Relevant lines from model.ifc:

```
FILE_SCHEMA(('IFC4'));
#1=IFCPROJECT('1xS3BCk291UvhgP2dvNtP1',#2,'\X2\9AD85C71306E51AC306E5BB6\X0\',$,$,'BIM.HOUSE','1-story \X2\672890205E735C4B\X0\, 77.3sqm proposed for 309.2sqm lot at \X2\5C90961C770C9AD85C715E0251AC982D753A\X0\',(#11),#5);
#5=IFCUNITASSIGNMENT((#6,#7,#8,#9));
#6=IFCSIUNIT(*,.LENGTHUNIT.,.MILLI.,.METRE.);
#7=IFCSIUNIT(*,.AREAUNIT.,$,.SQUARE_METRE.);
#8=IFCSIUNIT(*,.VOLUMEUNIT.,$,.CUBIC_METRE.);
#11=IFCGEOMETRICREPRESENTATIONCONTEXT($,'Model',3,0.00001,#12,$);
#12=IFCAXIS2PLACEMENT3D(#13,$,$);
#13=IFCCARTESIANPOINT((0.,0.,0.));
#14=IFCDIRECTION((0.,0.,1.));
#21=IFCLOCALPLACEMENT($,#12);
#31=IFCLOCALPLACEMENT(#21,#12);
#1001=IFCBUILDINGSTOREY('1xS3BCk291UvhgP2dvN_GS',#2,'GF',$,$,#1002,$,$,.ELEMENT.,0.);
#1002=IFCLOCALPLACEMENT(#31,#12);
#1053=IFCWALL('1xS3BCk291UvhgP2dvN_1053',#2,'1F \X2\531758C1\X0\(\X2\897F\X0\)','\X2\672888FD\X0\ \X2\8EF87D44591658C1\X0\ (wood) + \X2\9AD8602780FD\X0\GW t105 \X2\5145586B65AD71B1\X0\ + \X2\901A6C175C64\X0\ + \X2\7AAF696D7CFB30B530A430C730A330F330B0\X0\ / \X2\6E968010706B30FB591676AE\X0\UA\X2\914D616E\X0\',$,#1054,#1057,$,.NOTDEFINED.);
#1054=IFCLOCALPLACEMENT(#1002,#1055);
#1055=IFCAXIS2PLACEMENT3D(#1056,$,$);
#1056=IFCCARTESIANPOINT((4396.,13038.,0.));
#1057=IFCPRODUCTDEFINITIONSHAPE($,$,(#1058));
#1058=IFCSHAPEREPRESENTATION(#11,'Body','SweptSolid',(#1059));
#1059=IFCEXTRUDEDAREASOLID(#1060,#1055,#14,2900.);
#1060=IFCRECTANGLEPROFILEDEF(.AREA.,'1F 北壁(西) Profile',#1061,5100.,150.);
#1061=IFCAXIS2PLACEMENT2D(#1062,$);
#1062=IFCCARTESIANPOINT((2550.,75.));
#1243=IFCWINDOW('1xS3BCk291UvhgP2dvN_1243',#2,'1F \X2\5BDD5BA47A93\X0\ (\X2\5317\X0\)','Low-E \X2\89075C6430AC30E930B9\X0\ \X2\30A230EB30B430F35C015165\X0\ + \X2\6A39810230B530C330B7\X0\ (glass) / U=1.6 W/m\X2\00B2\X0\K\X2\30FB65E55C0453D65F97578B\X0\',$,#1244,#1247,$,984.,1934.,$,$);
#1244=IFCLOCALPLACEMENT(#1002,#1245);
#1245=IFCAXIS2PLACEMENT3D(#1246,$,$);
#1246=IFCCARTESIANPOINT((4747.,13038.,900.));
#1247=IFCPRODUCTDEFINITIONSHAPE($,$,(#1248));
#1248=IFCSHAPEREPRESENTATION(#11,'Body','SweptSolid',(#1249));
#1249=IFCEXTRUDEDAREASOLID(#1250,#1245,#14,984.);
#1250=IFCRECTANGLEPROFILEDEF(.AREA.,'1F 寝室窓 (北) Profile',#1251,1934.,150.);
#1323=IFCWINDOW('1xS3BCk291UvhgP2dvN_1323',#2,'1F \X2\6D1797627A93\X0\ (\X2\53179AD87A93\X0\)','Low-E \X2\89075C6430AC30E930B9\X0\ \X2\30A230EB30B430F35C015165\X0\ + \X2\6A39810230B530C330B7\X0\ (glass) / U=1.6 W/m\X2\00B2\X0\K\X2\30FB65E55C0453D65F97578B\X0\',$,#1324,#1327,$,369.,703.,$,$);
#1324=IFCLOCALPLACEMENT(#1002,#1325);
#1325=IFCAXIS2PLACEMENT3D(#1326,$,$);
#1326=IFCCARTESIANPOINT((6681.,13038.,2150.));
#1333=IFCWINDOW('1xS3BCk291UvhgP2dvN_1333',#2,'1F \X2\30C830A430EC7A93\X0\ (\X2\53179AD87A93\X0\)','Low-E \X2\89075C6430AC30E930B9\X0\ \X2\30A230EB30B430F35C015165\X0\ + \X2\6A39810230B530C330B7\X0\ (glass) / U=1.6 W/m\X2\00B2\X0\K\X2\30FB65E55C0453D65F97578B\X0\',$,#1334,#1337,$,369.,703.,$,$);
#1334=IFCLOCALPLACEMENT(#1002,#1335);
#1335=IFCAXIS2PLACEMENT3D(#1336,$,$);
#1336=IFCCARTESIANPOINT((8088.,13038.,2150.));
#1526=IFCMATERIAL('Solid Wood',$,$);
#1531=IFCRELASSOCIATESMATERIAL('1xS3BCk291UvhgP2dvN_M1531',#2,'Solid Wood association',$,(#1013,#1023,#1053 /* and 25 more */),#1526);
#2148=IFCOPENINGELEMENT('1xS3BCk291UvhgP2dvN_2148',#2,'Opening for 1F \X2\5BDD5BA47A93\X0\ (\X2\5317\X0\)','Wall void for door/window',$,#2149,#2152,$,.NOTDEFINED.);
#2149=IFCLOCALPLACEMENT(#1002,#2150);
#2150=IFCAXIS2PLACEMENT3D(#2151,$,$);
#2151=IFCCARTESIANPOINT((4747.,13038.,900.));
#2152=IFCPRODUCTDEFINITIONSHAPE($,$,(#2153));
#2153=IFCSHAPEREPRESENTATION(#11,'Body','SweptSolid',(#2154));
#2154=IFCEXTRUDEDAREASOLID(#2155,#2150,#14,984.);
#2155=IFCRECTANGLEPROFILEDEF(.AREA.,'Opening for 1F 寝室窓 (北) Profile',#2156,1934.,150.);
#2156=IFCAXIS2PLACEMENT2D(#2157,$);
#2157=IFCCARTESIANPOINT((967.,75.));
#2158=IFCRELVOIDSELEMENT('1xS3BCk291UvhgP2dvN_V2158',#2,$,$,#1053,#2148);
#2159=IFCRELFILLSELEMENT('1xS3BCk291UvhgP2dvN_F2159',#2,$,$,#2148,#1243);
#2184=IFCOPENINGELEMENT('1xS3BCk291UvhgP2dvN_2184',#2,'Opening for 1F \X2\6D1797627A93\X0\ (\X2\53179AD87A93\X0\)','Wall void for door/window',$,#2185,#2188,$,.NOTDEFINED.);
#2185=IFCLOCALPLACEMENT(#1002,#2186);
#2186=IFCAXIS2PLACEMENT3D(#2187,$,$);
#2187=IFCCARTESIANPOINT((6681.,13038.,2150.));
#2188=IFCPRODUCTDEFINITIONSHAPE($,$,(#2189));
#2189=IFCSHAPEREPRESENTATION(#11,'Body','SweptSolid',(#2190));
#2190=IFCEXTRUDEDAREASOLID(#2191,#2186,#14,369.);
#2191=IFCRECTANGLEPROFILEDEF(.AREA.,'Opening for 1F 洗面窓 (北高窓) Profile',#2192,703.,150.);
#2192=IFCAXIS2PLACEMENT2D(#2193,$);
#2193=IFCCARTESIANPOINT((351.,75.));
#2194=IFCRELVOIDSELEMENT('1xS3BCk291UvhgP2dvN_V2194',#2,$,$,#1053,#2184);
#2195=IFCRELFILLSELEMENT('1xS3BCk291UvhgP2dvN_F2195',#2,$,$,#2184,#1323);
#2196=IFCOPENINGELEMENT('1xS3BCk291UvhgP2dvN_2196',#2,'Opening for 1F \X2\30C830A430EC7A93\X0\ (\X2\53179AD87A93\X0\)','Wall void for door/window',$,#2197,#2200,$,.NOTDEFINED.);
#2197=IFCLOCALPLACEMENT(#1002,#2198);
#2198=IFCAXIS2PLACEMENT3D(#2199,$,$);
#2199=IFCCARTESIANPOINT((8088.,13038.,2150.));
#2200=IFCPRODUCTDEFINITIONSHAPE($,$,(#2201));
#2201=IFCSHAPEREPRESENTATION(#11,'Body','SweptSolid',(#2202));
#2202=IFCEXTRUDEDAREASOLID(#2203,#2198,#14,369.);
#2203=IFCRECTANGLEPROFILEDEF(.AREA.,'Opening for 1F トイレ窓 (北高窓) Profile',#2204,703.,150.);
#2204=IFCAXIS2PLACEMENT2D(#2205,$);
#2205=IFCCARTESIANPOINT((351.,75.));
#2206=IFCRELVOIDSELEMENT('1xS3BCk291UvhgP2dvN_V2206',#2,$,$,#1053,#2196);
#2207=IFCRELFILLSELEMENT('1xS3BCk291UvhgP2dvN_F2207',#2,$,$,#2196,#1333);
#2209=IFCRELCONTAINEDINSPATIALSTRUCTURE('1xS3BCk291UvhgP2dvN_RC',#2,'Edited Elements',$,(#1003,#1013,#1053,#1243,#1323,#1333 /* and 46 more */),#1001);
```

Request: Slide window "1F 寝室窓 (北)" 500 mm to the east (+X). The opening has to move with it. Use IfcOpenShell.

```python
import ifcopenshell
import ifcopenshell.api.geometry
import ifcopenshell.util.placement
import ifcopenshell.util.unit

model = ifcopenshell.open("model.ifc")
unit_scale = ifcopenshell.util.unit.calculate_unit_scale(model)

window = model.by_guid("1xS3BCk291UvhgP2dvN_1243")
opening = window.FillsVoids[0].RelatingOpeningElement
wall = opening.VoidsElements[0].RelatingBuildingElement

wall_matrix = ifcopenshell.util.placement.get_local_placement(wall.ObjectPlacement)
shift = wall_matrix[:3, 0] * 0.5 / unit_scale
before = ifcopenshell.util.placement.get_local_placement(window.ObjectPlacement)[:3, 3].copy()

# The window is not placed relative to its opening, so move both.
for product in (opening, window):
    matrix = ifcopenshell.util.placement.get_local_placement(product.ObjectPlacement)
    matrix[:3, 3] += shift
    ifcopenshell.api.geometry.edit_object_placement(model, product=product, matrix=matrix, is_si=False)

after = ifcopenshell.util.placement.get_local_placement(window.ObjectPlacement)[:3, 3]
print("window moved by", (after - before).round(3) + 0.0)

model.write("model_v2.ifc")
```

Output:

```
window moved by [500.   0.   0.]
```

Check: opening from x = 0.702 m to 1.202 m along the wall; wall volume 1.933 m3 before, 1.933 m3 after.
